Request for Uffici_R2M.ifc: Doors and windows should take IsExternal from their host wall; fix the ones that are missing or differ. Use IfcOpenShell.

First a look at what the model holds.

```python
import ifcopenshell
import ifcopenshell.util.element

model = ifcopenshell.open("Uffici_R2M.ifc")
print(model.schema)
seen = {}
for e in model.by_type("IfcDoor") + model.by_type("IfcWindow"):
    if not e.FillsVoids:
        continue
    host = e.FillsVoids[0].RelatingOpeningElement.VoidsElements[0].RelatingBuildingElement
    own = ifcopenshell.util.element.get_pset(e, f"Pset_{e.is_a()[3:].removesuffix('StandardCase')}Common", "IsExternal")
    wall = ifcopenshell.util.element.get_pset(host, "Pset_WallCommon", "IsExternal")
    seen[e.is_a(), own, wall] = seen.get((e.is_a(), own, wall), 0) + 1
for (cls, own, wall), count in sorted(seen.items(), key=str):
    print(count, cls, "IsExternal:", own, "| host wall:", wall)
```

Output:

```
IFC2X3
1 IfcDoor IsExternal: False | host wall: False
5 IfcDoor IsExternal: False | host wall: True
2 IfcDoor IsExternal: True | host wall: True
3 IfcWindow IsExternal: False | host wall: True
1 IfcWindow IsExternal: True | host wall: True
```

```python
import ifcopenshell
import ifcopenshell.api.pset
import ifcopenshell.util.element

model = ifcopenshell.open("Uffici_R2M.ifc")

count = 0
for ifc_class, pset_name in (("IfcDoor", "Pset_DoorCommon"), ("IfcWindow", "Pset_WindowCommon")):
    for e in model.by_type(ifc_class):
        if not e.FillsVoids:
            continue
        host = e.FillsVoids[0].RelatingOpeningElement.VoidsElements[0].RelatingBuildingElement
        external = ifcopenshell.util.element.get_pset(host, "Pset_WallCommon", "IsExternal")
        if external is None or ifcopenshell.util.element.get_pset(e, pset_name, "IsExternal") == external:
            continue
        pset = ifcopenshell.api.pset.add_pset(model, product=e, name=pset_name)
        ifcopenshell.api.pset.edit_pset(model, pset=pset, properties={"IsExternal": external})
        count += 1

print(count, "updated")

model.write("Uffici_R2M_v2.ifc")
```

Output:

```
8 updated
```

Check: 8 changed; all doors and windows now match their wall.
